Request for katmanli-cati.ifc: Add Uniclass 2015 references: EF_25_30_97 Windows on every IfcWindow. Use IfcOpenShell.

First a look at what the model holds.

```python
import ifcopenshell

model = ifcopenshell.open("katmanli-cati.ifc")
print(model.schema)
print("classifications:", [c.Name for c in model.by_type("IfcClassification")])
for ifc_class in ("IfcDoor", "IfcRoof", "IfcStair", "IfcWall", "IfcWindow"):
    print(ifc_class, len(model.by_type(ifc_class)))
```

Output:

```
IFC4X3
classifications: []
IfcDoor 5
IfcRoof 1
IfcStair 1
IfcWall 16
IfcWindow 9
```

```python
import ifcopenshell
import ifcopenshell.api.classification

model = ifcopenshell.open("katmanli-cati.ifc")

system = ifcopenshell.api.classification.add_classification(model, classification="Uniclass 2015")

codes = {
    "IfcWindow": ("EF_25_30_97", "Windows"),
}
for ifc_class, (code, name) in codes.items():
    products = model.by_type(ifc_class)
    ifcopenshell.api.classification.add_reference(
        model, products=products, classification=system, identification=code, name=name
    )
    print(code, len(products))

model.write("katmanli-cati_updated.ifc")
```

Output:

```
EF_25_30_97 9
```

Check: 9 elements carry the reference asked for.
